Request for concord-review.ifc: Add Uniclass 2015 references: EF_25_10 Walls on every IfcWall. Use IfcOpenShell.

First a look at what the model holds.

```python
import ifcopenshell

model = ifcopenshell.open("concord-review.ifc")
print(model.schema)
print("classifications:", [c.Name for c in model.by_type("IfcClassification")])
for ifc_class in ("IfcDoor", "IfcRoof", "IfcStair", "IfcWall", "IfcWindow"):
    print(ifc_class, len(model.by_type(ifc_class)))
```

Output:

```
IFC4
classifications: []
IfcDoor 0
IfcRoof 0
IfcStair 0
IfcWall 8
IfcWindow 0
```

```python
import ifcopenshell
import ifcopenshell.api.classification

model = ifcopenshell.open("concord-review.ifc")

system = ifcopenshell.api.classification.add_classification(model, classification="Uniclass 2015")

codes = {
    "IfcWall": ("EF_25_10", "Walls"),
}
for ifc_class, (code, name) in codes.items():
    products = model.by_type(ifc_class)
    ifcopenshell.api.classification.add_reference(
        model, products=products, classification=system, identification=code, name=name
    )
    print(code, len(products))

model.write("concord-review_edited.ifc")
```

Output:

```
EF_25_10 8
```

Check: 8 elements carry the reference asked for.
